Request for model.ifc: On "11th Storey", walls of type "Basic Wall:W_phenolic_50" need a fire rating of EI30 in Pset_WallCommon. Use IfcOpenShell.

First a look at what the model holds.

```python
import ifcopenshell
import ifcopenshell.util.element

model = ifcopenshell.open("model.ifc")
print(model.schema)
storey = next(s for s in model.by_type("IfcBuildingStorey") if s.Name == "11th Storey")
walls = [e for e in ifcopenshell.util.element.get_decomposition(storey) if e.is_a("IfcWall")]
seen = {}
for e in walls:
    element_type = ifcopenshell.util.element.get_type(e)
    key = (element_type.Name if element_type != e and element_type else None, ifcopenshell.util.element.get_pset(e, "Pset_WallCommon", "FireRating"))
    seen[key] = seen.get(key, 0) + 1
for (name, value), count in sorted(seen.items(), key=str):
    print(count, "x", name, "|", value)
```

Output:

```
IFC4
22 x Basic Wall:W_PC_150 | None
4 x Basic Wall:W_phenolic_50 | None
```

```python
import ifcopenshell
import ifcopenshell.api.pset
import ifcopenshell.util.element

model = ifcopenshell.open("model.ifc")

storey = next(s for s in model.by_type("IfcBuildingStorey") if s.Name == "11th Storey")
walls = [e for e in ifcopenshell.util.element.get_decomposition(storey) if e.is_a("IfcWall")]

count = 0
for e in walls:
    element_type = ifcopenshell.util.element.get_type(e)
    if element_type in (None, e) or element_type.Name != "Basic Wall:W_phenolic_50":
        continue
    # add_pset returns the element's existing set when there is one.
    pset = ifcopenshell.api.pset.add_pset(model, product=e, name="Pset_WallCommon")
    ifcopenshell.api.pset.edit_pset(model, pset=pset, properties={"FireRating": "EI30"})
    count += 1

print(count, "walls updated")

model.write("model_rev.ifc")
```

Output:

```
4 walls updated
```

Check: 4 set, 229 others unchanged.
